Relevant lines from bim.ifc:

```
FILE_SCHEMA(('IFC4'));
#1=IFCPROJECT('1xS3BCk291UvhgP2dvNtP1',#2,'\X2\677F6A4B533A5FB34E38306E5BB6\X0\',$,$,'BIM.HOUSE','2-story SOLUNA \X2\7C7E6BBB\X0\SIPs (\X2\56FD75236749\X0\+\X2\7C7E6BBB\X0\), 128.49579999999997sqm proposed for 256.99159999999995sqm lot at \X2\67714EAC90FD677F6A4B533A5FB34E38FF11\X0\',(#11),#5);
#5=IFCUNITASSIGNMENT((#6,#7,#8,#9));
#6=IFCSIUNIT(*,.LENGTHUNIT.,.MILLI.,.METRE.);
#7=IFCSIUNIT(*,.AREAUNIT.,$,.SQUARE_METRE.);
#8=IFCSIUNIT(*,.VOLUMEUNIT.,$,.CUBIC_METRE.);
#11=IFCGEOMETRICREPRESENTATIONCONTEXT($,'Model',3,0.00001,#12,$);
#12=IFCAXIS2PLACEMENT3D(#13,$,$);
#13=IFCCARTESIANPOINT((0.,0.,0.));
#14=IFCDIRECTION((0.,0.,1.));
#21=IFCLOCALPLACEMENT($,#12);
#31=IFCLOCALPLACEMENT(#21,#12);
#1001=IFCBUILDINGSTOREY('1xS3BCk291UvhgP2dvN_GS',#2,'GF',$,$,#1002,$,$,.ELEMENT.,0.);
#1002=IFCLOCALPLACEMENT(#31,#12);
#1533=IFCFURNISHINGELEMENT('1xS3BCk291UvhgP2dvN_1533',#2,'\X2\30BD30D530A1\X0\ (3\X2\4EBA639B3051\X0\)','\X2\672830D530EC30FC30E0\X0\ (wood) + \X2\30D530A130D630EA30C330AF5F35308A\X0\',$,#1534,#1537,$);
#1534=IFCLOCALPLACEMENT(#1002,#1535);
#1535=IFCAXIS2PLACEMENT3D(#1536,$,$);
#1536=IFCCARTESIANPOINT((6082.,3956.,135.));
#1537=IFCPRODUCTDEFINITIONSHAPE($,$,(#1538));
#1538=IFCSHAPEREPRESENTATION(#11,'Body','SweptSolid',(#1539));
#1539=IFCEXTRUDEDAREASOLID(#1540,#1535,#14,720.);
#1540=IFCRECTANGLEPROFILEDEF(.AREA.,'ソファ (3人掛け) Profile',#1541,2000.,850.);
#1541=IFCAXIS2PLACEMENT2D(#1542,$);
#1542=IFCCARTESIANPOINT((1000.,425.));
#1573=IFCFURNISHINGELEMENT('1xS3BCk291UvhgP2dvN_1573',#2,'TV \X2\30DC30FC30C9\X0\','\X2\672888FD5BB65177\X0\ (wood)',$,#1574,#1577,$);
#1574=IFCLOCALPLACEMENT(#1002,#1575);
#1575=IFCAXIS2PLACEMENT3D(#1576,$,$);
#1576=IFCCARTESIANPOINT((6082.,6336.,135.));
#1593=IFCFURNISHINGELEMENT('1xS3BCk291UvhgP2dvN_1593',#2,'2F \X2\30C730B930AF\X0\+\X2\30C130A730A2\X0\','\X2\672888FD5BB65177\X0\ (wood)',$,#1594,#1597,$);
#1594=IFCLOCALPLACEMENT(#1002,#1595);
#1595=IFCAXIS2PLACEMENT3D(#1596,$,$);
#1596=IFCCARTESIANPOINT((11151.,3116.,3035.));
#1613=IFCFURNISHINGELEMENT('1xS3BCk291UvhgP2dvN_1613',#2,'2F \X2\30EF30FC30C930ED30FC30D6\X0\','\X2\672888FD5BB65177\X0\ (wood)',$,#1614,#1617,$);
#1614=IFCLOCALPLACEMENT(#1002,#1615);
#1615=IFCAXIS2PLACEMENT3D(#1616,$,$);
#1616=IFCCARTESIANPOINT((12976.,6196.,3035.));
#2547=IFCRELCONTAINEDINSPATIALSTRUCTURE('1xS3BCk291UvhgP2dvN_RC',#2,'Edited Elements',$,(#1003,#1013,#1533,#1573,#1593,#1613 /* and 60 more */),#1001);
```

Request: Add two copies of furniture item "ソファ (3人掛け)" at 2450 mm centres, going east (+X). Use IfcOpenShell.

```python
import numpy as np
import ifcopenshell
import ifcopenshell.api.geometry
import ifcopenshell.api.root
import ifcopenshell.util.element
import ifcopenshell.util.placement

model = ifcopenshell.open("bim.ifc")


def reuse_history(source, copy):
    """copy_class also copies each property set's owner history, people and application; keep the originals."""
    for rel in copy.IsDefinedBy:
        if rel.is_a("IfcRelDefinesByProperties") and (history := rel.RelatingPropertyDefinition.OwnerHistory):
            rel.RelatingPropertyDefinition.OwnerHistory = source.OwnerHistory
            ifcopenshell.util.element.remove_deep2(model, history)


source = model.by_guid("1xS3BCk291UvhgP2dvN_1533")
base = ifcopenshell.util.placement.get_local_placement(source.ObjectPlacement)
step = np.array([1.0, 0.0, 0.0]) * 2450.0

for i in range(1, 3):
    copy = ifcopenshell.api.root.copy_class(model, product=source)
    copy.Representation = ifcopenshell.util.element.copy_deep(
        model, source.Representation, exclude=["IfcGeometricRepresentationContext", "IfcRepresentationMap"]
    )
    reuse_history(source, copy)
    matrix = base.copy()
    matrix[:3, 3] += i * step
    print("added at", matrix[:3, 3].round(3) + 0.0)
    ifcopenshell.api.geometry.edit_object_placement(model, product=copy, matrix=matrix, is_si=False)

model.write("bim_updated.ifc")
```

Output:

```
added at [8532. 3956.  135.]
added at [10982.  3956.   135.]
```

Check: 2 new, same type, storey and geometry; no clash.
